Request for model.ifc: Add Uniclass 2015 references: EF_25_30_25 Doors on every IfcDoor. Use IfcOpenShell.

First a look at what the model holds.

```python
import ifcopenshell

model = ifcopenshell.open("model.ifc")
print(model.schema)
print("classifications:", [c.Name for c in model.by_type("IfcClassification")])
for ifc_class in ("IfcDoor", "IfcRoof", "IfcStair", "IfcWall", "IfcWindow"):
    print(ifc_class, len(model.by_type(ifc_class)))
```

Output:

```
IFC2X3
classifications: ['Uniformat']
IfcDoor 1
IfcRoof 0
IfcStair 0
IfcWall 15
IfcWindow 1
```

```python
import ifcopenshell
import ifcopenshell.api.classification

model = ifcopenshell.open("model.ifc")

# IFC2X3 requires Source and Edition and has no link from the project to the system.
system = model.create_entity("IfcClassification", Source="NBS", Edition="2015", Name="Uniclass 2015")

codes = {
    "IfcDoor": ("EF_25_30_25", "Doors"),
}
for ifc_class, (code, name) in codes.items():
    products = model.by_type(ifc_class)
    ifcopenshell.api.classification.add_reference(
        model, products=products, classification=system, identification=code, name=name
    )
    print(code, len(products))

model.write("model_edited.ifc")
```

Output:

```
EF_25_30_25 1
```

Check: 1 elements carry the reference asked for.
